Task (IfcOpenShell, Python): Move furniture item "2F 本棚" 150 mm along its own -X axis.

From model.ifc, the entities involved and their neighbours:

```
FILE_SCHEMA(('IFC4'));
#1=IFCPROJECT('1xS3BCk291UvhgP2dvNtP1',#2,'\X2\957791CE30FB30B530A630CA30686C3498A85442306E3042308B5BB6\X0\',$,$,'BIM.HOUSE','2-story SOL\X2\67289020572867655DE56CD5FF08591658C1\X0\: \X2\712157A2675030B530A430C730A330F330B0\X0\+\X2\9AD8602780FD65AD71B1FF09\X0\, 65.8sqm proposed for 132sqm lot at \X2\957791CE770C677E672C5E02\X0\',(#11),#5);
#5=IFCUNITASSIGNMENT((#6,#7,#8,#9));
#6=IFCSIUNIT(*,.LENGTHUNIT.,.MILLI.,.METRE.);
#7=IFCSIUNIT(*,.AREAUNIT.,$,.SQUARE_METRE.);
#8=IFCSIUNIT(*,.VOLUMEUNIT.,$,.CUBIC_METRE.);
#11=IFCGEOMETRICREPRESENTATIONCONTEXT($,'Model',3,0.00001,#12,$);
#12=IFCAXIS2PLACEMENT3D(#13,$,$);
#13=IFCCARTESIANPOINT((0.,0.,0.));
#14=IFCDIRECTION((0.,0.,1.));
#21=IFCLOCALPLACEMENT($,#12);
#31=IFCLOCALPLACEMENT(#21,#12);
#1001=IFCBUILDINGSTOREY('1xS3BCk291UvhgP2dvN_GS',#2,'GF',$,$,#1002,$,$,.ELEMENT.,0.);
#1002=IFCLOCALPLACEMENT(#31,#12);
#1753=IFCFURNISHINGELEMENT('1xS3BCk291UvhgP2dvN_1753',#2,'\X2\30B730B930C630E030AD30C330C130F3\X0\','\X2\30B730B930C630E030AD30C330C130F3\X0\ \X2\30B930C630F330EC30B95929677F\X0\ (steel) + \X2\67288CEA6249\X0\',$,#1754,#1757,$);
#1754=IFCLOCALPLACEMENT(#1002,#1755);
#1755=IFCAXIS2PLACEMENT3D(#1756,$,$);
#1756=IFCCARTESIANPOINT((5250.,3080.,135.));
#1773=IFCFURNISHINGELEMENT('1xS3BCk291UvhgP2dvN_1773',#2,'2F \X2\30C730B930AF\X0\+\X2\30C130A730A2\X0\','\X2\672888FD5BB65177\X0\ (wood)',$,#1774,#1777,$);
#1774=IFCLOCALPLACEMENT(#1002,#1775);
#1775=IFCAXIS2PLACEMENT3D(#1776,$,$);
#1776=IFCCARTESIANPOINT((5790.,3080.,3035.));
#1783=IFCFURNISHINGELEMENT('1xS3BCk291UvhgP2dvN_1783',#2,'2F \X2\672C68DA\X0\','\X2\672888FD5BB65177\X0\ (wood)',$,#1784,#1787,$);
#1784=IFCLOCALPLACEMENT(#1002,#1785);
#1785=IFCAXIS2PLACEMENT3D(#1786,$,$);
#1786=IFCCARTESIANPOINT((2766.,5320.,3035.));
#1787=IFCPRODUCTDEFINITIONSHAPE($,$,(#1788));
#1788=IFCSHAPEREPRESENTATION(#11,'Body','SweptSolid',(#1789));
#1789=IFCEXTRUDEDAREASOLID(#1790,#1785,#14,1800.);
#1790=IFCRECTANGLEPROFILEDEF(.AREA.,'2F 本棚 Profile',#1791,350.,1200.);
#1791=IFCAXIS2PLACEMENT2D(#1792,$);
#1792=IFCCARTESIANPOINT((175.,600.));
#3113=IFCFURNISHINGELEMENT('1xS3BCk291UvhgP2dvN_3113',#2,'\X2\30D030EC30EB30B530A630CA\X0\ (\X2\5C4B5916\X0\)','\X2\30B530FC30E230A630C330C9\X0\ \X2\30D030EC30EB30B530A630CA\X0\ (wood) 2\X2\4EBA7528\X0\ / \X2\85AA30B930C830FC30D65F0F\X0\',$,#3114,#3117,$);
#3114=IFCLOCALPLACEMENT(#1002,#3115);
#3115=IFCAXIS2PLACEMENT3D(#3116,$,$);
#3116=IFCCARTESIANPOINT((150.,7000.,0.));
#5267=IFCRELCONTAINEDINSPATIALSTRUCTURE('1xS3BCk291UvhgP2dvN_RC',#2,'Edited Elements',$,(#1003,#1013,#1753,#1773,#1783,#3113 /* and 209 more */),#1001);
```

```python
import ifcopenshell
import ifcopenshell.api.geometry
import ifcopenshell.util.placement
import ifcopenshell.util.unit

model = ifcopenshell.open("model.ifc")
unit_scale = ifcopenshell.util.unit.calculate_unit_scale(model)

item = model.by_id(1783)
matrix = ifcopenshell.util.placement.get_local_placement(item.ObjectPlacement)
matrix[:3, 3] -= matrix[:3, 0] * 0.15 / unit_scale
ifcopenshell.api.geometry.edit_object_placement(model, product=item, matrix=matrix, is_si=False)

print(ifcopenshell.util.placement.get_local_placement(item.ObjectPlacement).round(3) + 0.0)

model.write("model_edited.ifc")
```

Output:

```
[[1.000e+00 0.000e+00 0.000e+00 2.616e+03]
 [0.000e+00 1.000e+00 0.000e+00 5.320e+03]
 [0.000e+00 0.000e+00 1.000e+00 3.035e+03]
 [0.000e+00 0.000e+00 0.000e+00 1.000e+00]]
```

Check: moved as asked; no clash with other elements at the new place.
